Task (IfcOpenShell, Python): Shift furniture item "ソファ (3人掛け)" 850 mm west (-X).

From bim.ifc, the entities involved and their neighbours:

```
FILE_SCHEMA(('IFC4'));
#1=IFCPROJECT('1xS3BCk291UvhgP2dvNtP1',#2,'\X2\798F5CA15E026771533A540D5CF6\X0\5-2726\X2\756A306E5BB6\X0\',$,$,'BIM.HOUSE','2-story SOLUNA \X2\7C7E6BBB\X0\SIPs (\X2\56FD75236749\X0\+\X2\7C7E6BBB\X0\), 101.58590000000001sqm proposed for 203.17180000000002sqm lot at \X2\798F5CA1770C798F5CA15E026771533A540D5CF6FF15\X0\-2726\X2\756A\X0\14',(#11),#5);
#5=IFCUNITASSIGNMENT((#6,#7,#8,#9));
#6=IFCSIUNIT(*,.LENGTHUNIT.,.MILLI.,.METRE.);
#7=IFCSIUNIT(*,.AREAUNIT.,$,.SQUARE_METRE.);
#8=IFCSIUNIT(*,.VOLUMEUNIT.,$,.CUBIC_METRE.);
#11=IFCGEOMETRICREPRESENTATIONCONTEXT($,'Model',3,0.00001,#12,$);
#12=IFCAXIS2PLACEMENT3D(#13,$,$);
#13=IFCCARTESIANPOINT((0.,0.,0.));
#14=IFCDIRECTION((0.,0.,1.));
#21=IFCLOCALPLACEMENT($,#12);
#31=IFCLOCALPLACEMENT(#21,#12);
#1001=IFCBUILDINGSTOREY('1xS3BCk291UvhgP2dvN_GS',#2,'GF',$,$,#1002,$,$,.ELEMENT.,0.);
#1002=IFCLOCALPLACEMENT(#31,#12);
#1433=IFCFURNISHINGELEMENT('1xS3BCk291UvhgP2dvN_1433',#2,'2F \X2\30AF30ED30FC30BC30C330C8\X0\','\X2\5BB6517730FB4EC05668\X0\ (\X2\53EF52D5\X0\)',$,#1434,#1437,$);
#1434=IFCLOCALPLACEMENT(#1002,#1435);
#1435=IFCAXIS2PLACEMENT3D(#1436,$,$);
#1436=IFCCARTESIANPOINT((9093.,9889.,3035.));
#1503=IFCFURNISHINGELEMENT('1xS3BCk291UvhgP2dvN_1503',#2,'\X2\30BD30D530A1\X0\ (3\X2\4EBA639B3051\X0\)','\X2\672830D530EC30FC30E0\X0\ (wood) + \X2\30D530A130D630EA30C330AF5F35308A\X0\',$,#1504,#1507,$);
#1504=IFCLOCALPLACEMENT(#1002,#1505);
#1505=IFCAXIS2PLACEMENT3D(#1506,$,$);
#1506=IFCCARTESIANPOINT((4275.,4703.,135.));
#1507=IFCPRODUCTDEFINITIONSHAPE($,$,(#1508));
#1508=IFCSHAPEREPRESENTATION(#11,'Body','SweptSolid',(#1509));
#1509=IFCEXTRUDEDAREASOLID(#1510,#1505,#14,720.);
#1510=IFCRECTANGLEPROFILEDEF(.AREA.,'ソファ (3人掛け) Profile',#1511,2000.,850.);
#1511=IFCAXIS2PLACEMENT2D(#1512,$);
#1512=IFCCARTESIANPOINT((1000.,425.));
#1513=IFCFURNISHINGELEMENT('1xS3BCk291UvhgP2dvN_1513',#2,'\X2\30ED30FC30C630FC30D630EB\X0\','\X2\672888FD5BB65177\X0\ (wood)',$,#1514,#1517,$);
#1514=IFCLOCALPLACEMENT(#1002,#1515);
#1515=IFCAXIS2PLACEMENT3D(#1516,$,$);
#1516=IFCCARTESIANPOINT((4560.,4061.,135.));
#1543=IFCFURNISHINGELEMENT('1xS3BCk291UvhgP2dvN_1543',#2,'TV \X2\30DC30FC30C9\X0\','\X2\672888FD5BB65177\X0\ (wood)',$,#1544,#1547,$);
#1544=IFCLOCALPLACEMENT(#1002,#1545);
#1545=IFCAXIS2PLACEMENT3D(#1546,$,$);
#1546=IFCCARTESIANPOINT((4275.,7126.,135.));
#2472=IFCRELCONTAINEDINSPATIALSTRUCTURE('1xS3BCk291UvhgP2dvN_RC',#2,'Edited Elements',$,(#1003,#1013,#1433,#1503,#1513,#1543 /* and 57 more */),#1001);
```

```python
import ifcopenshell
import ifcopenshell.api.geometry
import ifcopenshell.util.placement
import ifcopenshell.util.unit

model = ifcopenshell.open("bim.ifc")
unit_scale = ifcopenshell.util.unit.calculate_unit_scale(model)

item = model.by_guid("1xS3BCk291UvhgP2dvN_1503")
matrix = ifcopenshell.util.placement.get_local_placement(item.ObjectPlacement)
matrix[0, 3] -= 0.85 / unit_scale
ifcopenshell.api.geometry.edit_object_placement(model, product=item, matrix=matrix, is_si=False)

print(ifcopenshell.util.placement.get_local_placement(item.ObjectPlacement).round(3) + 0.0)

model.write("bim_v2.ifc")
```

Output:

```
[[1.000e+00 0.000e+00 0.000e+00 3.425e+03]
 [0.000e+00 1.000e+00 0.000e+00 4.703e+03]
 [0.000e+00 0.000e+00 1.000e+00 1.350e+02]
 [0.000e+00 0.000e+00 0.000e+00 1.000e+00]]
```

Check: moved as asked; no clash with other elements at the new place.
